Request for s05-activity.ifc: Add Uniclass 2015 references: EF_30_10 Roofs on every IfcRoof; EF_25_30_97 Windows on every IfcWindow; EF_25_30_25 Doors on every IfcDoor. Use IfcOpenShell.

First a look at what the model holds.

```python
import ifcopenshell

model = ifcopenshell.open("s05-activity.ifc")
print(model.schema)
print("classifications:", [c.Name for c in model.by_type("IfcClassification")])
for ifc_class in ("IfcDoor", "IfcRoof", "IfcStair", "IfcWall", "IfcWindow"):
    print(ifc_class, len(model.by_type(ifc_class)))
```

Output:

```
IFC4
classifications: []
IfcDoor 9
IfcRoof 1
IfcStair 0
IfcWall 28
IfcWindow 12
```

```python
import ifcopenshell
import ifcopenshell.api.classification

model = ifcopenshell.open("s05-activity.ifc")

system = ifcopenshell.api.classification.add_classification(model, classification="Uniclass 2015")

codes = {
    "IfcRoof": ("EF_30_10", "Roofs"),
    "IfcWindow": ("EF_25_30_97", "Windows"),
    "IfcDoor": ("EF_25_30_25", "Doors"),
}
for ifc_class, (code, name) in codes.items():
    products = model.by_type(ifc_class)
    ifcopenshell.api.classification.add_reference(
        model, products=products, classification=system, identification=code, name=name
    )
    print(code, len(products))

model.write("s05-activity_rev.ifc")
```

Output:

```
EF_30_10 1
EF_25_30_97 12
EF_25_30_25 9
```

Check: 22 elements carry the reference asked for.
